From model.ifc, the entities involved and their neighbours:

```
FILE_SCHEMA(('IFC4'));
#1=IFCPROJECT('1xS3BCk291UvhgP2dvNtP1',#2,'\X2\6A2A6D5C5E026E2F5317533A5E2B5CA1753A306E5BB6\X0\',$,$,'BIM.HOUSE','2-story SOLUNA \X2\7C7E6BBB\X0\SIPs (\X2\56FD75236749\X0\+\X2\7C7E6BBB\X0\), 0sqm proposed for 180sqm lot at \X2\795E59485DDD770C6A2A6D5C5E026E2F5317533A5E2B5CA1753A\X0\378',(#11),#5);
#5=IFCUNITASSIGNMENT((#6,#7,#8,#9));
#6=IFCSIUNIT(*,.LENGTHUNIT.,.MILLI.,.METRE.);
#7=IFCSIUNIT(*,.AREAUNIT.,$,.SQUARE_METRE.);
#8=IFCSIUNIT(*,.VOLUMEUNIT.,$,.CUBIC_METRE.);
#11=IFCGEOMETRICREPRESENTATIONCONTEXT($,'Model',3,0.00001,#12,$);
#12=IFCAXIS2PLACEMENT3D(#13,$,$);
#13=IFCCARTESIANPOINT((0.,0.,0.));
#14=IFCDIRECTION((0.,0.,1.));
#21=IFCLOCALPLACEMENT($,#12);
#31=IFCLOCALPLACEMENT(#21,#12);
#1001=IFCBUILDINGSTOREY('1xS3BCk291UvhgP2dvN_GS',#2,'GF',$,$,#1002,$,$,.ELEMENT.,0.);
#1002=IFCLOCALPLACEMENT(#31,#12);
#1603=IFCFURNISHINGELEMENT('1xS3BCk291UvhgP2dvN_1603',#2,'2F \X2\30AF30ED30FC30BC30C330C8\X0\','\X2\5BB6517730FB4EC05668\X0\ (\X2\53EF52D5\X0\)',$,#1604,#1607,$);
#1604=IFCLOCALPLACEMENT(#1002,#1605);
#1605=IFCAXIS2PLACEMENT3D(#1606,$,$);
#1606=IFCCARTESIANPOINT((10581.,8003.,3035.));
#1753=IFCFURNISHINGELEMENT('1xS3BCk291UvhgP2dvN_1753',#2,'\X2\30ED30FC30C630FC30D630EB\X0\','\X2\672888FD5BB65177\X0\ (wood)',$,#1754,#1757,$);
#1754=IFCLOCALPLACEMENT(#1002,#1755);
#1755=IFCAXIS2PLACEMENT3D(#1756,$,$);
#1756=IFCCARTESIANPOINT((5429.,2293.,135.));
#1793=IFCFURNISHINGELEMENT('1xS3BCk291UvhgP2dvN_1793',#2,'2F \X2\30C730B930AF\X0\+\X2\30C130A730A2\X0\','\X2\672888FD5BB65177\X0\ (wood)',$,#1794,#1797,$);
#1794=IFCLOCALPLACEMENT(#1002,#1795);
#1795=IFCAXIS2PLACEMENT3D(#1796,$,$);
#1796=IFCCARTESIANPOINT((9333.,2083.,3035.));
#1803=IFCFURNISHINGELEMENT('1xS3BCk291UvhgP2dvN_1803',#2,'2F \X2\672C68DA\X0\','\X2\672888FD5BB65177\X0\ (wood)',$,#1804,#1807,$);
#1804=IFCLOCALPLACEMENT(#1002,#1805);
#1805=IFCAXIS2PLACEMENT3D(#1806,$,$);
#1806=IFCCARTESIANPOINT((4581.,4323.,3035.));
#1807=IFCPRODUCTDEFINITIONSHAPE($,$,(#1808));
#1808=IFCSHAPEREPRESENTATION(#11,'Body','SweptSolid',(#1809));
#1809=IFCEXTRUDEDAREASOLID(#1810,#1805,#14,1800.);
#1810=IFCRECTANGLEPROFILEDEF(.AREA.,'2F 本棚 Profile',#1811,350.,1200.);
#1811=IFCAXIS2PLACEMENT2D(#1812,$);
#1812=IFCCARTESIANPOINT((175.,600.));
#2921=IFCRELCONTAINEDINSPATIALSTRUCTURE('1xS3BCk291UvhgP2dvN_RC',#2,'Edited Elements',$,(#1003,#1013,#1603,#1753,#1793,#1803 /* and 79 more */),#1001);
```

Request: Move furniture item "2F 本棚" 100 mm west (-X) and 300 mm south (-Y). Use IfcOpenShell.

```python
import ifcopenshell
import ifcopenshell.api.geometry
import ifcopenshell.util.placement
import ifcopenshell.util.unit

model = ifcopenshell.open("model.ifc")
unit_scale = ifcopenshell.util.unit.calculate_unit_scale(model)

item = model.by_guid("1xS3BCk291UvhgP2dvN_1803")
matrix = ifcopenshell.util.placement.get_local_placement(item.ObjectPlacement)
matrix[0, 3] -= 0.1 / unit_scale
matrix[1, 3] -= 0.3 / unit_scale
ifcopenshell.api.geometry.edit_object_placement(model, product=item, matrix=matrix, is_si=False)

print(ifcopenshell.util.placement.get_local_placement(item.ObjectPlacement).round(3) + 0.0)

model.write("model_edited.ifc")
```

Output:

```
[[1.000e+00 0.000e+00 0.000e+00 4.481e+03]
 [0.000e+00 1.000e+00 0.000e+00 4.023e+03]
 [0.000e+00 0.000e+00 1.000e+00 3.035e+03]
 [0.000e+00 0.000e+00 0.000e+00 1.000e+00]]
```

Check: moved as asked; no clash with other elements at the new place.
